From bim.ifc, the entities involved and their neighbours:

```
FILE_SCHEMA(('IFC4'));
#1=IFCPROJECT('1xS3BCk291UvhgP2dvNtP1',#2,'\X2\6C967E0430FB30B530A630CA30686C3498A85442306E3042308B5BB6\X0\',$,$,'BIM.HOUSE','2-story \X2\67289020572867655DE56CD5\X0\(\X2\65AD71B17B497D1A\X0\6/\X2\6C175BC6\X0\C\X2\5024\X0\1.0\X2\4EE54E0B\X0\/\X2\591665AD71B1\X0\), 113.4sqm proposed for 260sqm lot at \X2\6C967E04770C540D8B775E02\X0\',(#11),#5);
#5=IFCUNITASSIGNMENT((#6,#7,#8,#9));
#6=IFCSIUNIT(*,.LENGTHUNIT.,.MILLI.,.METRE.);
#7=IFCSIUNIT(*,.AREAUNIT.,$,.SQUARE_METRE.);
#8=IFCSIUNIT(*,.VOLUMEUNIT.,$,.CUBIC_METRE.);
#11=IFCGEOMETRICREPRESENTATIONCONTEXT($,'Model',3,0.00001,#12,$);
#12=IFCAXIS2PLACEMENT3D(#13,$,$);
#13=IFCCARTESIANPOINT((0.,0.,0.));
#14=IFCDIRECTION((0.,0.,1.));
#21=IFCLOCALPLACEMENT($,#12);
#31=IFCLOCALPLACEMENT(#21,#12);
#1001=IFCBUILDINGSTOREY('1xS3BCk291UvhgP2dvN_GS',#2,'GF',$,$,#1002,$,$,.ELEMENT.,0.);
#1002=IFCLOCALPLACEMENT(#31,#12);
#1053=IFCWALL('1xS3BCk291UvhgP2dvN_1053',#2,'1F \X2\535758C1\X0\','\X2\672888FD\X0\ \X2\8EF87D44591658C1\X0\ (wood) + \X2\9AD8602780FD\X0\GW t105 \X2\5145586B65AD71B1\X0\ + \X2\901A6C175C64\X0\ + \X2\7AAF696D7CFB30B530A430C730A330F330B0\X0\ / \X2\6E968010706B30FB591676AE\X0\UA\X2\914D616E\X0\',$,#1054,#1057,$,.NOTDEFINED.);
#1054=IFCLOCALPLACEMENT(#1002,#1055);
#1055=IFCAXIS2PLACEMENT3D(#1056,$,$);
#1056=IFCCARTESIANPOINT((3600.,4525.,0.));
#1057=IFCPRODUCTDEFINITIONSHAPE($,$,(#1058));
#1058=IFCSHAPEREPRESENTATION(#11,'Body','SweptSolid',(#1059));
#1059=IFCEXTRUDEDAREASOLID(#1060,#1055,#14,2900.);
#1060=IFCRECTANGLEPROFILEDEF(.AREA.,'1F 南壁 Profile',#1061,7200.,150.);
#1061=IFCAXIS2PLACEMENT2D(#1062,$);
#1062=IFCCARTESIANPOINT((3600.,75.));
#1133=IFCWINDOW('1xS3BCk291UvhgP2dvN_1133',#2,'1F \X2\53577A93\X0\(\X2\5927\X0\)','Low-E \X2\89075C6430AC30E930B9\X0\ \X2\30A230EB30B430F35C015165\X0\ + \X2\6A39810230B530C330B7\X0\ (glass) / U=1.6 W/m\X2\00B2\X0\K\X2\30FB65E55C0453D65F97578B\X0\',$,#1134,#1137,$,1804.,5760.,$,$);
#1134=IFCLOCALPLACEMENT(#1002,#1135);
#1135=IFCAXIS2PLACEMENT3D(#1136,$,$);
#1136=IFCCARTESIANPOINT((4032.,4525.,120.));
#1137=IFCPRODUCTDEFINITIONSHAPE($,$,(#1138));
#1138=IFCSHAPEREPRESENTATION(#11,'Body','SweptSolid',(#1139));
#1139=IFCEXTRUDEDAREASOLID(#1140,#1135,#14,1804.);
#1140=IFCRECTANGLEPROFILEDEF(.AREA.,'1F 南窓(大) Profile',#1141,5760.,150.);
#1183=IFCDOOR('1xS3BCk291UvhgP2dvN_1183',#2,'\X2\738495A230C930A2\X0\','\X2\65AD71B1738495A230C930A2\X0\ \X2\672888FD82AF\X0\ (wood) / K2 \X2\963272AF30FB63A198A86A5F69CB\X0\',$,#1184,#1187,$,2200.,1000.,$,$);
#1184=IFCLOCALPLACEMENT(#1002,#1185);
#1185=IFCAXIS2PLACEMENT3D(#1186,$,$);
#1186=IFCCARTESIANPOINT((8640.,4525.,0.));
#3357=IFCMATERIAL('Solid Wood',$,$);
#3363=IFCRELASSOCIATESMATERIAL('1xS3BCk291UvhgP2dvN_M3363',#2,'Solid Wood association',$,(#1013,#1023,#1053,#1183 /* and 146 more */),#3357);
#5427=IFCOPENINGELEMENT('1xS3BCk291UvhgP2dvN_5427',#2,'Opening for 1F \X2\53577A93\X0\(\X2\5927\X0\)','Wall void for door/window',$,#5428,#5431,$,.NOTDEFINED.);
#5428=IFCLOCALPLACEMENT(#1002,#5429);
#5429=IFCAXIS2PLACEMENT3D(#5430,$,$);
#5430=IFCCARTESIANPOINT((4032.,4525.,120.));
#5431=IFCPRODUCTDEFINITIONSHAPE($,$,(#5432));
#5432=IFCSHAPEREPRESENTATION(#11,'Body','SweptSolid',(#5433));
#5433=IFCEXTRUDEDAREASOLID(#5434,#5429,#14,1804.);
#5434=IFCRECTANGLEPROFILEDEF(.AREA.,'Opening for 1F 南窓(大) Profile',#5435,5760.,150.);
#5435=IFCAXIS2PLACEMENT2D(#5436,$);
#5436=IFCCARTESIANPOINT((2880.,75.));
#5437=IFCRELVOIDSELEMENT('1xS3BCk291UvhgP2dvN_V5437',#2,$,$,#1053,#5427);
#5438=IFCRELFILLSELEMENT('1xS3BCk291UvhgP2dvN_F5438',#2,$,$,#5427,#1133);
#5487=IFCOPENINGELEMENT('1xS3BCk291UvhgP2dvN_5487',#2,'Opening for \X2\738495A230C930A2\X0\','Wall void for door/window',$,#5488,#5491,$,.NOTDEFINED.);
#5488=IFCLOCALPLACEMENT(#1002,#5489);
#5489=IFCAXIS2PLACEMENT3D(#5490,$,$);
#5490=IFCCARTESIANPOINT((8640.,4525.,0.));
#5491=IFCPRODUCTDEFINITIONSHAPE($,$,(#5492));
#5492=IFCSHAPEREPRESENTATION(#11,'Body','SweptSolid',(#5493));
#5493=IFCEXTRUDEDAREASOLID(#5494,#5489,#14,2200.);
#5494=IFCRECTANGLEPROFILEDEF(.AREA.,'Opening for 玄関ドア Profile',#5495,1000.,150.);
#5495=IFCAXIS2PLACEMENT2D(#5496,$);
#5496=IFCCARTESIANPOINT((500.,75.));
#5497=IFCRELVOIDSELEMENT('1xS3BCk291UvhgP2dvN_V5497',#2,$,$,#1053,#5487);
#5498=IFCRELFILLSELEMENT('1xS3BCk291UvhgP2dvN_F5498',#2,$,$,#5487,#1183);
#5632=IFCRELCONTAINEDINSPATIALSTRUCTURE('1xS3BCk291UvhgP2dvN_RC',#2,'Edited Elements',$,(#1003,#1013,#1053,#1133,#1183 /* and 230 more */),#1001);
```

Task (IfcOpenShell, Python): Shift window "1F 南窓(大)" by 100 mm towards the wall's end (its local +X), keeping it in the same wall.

```python
import ifcopenshell
import ifcopenshell.api.geometry
import ifcopenshell.util.placement

model = ifcopenshell.open("bim.ifc")

window = model.by_guid("1xS3BCk291UvhgP2dvN_1133")
opening = window.FillsVoids[0].RelatingOpeningElement
wall = opening.VoidsElements[0].RelatingBuildingElement

wall_matrix = ifcopenshell.util.placement.get_local_placement(wall.ObjectPlacement)
shift = wall_matrix[:3, 0] * 100.0
before = ifcopenshell.util.placement.get_local_placement(window.ObjectPlacement)[:3, 3].copy()

# The window is not placed relative to its opening, so move both.
for product in (opening, window):
    matrix = ifcopenshell.util.placement.get_local_placement(product.ObjectPlacement)
    matrix[:3, 3] += shift
    ifcopenshell.api.geometry.edit_object_placement(model, product=product, matrix=matrix, is_si=False)

after = ifcopenshell.util.placement.get_local_placement(window.ObjectPlacement)[:3, 3]
print("window moved by", (after - before).round(3) + 0.0)

model.write("bim_edited.ifc")
```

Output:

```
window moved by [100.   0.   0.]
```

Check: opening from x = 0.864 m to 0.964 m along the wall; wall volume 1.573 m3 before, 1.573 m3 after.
